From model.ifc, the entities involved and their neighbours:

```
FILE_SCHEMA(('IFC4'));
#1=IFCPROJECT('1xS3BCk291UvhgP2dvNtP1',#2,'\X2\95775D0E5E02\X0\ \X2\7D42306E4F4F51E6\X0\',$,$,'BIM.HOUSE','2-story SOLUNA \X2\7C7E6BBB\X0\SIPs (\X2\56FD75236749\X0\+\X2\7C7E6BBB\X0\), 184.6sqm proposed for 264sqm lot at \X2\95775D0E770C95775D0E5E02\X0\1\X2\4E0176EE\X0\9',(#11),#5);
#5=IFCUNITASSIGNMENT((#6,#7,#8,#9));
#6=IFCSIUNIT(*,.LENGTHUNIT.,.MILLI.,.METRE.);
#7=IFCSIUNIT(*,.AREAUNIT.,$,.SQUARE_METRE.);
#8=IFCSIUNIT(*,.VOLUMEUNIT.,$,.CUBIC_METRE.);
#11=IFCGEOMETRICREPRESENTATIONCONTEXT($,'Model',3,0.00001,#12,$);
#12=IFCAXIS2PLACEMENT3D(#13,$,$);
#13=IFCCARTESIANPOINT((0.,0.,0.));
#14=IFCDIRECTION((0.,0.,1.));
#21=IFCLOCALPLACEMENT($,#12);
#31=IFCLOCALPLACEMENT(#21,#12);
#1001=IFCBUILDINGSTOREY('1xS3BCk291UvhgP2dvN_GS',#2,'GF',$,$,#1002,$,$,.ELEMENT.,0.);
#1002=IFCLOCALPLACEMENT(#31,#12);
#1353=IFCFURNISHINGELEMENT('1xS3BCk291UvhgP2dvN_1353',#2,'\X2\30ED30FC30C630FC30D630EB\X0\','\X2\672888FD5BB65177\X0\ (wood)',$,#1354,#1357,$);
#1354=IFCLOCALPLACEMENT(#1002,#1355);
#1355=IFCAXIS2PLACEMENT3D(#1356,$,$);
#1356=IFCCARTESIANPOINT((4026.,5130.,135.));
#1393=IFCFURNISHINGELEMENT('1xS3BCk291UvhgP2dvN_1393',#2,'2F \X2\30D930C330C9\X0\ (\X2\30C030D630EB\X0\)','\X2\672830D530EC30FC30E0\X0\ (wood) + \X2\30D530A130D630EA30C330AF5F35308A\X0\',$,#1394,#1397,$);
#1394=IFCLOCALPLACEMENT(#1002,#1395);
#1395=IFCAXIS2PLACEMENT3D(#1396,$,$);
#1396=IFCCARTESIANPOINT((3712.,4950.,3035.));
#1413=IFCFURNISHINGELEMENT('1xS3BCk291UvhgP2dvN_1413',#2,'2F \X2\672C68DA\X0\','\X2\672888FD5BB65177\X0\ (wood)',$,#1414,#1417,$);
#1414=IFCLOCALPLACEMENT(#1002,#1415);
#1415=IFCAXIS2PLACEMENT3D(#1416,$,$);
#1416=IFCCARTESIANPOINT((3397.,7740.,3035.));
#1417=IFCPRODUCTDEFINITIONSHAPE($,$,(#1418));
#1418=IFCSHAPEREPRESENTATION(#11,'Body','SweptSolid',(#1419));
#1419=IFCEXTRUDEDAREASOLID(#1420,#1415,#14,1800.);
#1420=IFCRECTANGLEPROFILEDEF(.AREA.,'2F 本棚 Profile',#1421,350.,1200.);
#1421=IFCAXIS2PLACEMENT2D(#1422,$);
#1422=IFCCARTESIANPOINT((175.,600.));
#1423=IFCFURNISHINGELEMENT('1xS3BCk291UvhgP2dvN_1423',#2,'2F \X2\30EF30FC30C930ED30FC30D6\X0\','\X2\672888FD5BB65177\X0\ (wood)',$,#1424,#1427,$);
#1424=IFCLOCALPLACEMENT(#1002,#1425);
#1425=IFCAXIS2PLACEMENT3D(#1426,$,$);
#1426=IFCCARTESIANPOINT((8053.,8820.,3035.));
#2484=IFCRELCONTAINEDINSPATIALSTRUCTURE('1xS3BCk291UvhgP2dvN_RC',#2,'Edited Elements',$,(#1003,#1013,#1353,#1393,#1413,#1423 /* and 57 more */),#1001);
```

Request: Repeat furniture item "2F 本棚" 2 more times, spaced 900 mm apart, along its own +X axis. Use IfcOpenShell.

```python
import ifcopenshell
import ifcopenshell.api.geometry
import ifcopenshell.api.root
import ifcopenshell.util.element
import ifcopenshell.util.placement

model = ifcopenshell.open("model.ifc")


def reuse_history(source, copy):
    """copy_class also copies each property set's owner history, people and application; keep the originals."""
    for rel in copy.IsDefinedBy:
        if rel.is_a("IfcRelDefinesByProperties") and (history := rel.RelatingPropertyDefinition.OwnerHistory):
            rel.RelatingPropertyDefinition.OwnerHistory = source.OwnerHistory
            ifcopenshell.util.element.remove_deep2(model, history)


source = model.by_guid("1xS3BCk291UvhgP2dvN_1413")
base = ifcopenshell.util.placement.get_local_placement(source.ObjectPlacement)
step = base[:3, 0] * 900.0

for i in range(1, 3):
    copy = ifcopenshell.api.root.copy_class(model, product=source)
    copy.Representation = ifcopenshell.util.element.copy_deep(
        model, source.Representation, exclude=["IfcGeometricRepresentationContext", "IfcRepresentationMap"]
    )
    reuse_history(source, copy)
    matrix = base.copy()
    matrix[:3, 3] += i * step
    print("added at", matrix[:3, 3].round(3) + 0.0)
    ifcopenshell.api.geometry.edit_object_placement(model, product=copy, matrix=matrix, is_si=False)

model.write("model-out.ifc")
```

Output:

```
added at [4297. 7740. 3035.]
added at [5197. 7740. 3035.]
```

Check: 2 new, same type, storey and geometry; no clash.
